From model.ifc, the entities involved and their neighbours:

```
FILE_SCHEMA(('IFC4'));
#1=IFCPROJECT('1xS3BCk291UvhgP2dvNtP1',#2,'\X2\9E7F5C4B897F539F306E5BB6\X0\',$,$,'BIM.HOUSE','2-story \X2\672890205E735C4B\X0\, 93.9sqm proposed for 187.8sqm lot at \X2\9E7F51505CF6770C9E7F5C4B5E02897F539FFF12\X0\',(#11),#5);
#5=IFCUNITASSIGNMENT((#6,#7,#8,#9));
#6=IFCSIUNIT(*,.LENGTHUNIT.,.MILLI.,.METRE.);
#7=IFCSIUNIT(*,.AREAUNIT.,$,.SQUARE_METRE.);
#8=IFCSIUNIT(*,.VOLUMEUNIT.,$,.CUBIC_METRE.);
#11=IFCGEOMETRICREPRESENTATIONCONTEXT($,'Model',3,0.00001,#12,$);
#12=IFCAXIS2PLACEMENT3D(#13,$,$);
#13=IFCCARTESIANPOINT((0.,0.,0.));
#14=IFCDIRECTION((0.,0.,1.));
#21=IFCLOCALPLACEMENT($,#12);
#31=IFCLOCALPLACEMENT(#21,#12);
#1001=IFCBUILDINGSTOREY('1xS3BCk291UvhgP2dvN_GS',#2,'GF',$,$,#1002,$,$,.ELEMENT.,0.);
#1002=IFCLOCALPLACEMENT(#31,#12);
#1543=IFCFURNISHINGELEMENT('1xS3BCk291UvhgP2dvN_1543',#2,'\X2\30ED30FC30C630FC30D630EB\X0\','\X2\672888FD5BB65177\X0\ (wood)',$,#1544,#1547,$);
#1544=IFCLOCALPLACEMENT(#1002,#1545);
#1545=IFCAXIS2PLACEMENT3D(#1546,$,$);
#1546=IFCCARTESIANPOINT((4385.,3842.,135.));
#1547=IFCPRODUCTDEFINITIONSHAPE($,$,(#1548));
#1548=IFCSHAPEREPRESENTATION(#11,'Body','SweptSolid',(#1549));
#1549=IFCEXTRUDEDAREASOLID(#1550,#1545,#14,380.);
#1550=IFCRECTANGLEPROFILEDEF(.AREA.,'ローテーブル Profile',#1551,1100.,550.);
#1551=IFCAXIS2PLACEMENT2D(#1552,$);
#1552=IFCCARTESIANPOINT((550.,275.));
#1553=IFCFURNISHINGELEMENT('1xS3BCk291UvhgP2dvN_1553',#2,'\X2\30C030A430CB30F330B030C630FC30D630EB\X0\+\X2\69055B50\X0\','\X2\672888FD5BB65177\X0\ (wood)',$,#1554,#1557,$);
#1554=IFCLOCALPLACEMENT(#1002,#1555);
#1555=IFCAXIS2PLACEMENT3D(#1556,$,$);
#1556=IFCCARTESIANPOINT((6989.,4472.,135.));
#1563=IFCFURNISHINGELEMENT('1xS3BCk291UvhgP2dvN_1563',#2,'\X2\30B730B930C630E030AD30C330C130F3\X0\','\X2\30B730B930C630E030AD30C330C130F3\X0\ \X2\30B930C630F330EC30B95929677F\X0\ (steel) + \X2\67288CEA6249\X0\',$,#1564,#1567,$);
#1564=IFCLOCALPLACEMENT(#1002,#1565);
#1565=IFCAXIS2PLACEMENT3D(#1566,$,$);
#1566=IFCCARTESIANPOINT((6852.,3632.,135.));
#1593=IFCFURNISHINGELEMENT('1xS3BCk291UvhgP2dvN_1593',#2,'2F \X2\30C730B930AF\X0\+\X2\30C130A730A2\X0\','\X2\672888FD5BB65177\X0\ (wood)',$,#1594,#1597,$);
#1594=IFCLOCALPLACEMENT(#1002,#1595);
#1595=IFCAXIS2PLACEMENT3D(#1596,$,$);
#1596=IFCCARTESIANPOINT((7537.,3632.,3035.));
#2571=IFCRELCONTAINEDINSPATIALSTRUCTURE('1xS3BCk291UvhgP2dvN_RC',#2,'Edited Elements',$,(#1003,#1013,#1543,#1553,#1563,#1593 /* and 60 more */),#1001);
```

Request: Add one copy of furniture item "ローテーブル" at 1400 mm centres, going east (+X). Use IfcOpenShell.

```python
import numpy as np
import ifcopenshell
import ifcopenshell.api.geometry
import ifcopenshell.api.root
import ifcopenshell.util.element
import ifcopenshell.util.placement
import ifcopenshell.util.unit

model = ifcopenshell.open("model.ifc")
unit_scale = ifcopenshell.util.unit.calculate_unit_scale(model)


def reuse_history(source, copy):
    """copy_class also copies each property set's owner history, people and application; keep the originals."""
    for rel in copy.IsDefinedBy:
        if rel.is_a("IfcRelDefinesByProperties") and (history := rel.RelatingPropertyDefinition.OwnerHistory):
            rel.RelatingPropertyDefinition.OwnerHistory = source.OwnerHistory
            ifcopenshell.util.element.remove_deep2(model, history)


source = model.by_guid("1xS3BCk291UvhgP2dvN_1543")
base = ifcopenshell.util.placement.get_local_placement(source.ObjectPlacement)
step = np.array([1.0, 0.0, 0.0]) * 1.4 / unit_scale

for i in range(1, 2):
    copy = ifcopenshell.api.root.copy_class(model, product=source)
    copy.Representation = ifcopenshell.util.element.copy_deep(
        model, source.Representation, exclude=["IfcGeometricRepresentationContext", "IfcRepresentationMap"]
    )
    reuse_history(source, copy)
    matrix = base.copy()
    matrix[:3, 3] += i * step
    print("added at", matrix[:3, 3].round(3) + 0.0)
    ifcopenshell.api.geometry.edit_object_placement(model, product=copy, matrix=matrix, is_si=False)

model.write("model_edited.ifc")
```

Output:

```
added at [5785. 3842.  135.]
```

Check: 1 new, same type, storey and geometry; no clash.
